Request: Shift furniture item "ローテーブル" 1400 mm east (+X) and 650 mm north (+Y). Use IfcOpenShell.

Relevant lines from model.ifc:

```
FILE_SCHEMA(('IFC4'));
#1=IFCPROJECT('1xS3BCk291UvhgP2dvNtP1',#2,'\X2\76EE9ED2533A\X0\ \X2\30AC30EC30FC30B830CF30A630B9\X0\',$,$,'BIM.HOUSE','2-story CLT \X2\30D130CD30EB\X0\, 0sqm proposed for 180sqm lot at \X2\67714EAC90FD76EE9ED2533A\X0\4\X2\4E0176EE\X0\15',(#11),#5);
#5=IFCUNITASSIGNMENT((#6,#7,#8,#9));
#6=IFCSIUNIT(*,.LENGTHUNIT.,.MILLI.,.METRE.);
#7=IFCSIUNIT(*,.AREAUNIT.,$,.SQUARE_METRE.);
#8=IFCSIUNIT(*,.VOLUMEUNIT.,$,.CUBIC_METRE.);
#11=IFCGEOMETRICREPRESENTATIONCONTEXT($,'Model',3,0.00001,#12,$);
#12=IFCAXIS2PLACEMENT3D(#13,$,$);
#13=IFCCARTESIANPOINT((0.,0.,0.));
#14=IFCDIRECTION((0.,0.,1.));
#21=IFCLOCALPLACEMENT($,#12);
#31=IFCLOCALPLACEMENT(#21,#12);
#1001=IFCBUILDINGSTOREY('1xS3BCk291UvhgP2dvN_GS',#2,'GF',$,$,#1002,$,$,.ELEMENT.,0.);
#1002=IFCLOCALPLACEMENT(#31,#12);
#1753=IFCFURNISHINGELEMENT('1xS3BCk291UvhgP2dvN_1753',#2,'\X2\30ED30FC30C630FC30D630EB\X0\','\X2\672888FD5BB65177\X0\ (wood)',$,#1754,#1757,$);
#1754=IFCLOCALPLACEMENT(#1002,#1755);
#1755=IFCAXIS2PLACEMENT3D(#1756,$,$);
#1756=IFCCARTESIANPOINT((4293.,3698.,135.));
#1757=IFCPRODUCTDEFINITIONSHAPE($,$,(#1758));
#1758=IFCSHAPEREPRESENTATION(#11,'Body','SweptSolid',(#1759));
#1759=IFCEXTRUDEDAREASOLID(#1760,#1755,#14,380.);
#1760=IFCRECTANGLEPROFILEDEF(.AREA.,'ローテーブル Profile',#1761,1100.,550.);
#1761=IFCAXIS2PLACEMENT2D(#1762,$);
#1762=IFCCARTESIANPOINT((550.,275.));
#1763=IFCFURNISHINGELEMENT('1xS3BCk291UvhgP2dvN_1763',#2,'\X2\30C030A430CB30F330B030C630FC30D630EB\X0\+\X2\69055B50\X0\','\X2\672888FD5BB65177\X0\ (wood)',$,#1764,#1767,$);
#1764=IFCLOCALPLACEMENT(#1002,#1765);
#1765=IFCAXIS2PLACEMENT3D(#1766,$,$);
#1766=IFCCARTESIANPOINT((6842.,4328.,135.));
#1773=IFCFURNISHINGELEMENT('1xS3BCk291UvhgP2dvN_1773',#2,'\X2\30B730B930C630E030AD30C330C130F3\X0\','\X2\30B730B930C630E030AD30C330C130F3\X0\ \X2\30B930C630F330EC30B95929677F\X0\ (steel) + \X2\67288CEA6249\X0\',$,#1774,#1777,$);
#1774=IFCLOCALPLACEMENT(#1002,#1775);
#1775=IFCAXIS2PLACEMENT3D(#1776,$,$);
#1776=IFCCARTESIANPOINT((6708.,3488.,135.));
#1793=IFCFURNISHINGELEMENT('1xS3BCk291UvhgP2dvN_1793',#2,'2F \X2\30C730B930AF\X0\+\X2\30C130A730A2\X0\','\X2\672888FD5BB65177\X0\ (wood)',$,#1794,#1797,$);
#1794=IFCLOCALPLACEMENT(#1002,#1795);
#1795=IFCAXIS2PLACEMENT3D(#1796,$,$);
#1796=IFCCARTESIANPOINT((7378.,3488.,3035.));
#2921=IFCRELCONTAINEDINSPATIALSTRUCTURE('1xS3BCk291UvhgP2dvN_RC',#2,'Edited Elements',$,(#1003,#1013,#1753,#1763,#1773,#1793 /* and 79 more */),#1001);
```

```python
import ifcopenshell
import ifcopenshell.api.geometry
import ifcopenshell.util.placement
import ifcopenshell.util.unit

model = ifcopenshell.open("model.ifc")
unit_scale = ifcopenshell.util.unit.calculate_unit_scale(model)

item = model.by_guid("1xS3BCk291UvhgP2dvN_1753")
matrix = ifcopenshell.util.placement.get_local_placement(item.ObjectPlacement)
matrix[0, 3] += 1.4 / unit_scale
matrix[1, 3] += 0.65 / unit_scale
ifcopenshell.api.geometry.edit_object_placement(model, product=item, matrix=matrix, is_si=False)

print(ifcopenshell.util.placement.get_local_placement(item.ObjectPlacement).round(3) + 0.0)

model.write("model_v2.ifc")
```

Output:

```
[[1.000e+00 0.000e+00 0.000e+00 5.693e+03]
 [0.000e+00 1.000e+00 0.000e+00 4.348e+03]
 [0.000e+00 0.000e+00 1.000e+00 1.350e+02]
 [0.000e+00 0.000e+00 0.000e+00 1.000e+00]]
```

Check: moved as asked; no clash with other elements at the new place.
